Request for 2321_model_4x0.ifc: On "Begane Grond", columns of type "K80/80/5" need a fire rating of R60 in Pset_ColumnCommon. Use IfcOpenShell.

First a look at what the model holds.

```python
import ifcopenshell
import ifcopenshell.util.element

model = ifcopenshell.open("2321_model_4x0.ifc")
print(model.schema)
storey = next(s for s in model.by_type("IfcBuildingStorey") if s.Name == "Begane Grond")
columns = [e for e in ifcopenshell.util.element.get_decomposition(storey) if e.is_a("IfcColumn")]
seen = {}
for e in columns:
    element_type = ifcopenshell.util.element.get_type(e)
    key = (element_type.Name if element_type != e and element_type else None, ifcopenshell.util.element.get_pset(e, "Pset_ColumnCommon", "FireRating"))
    seen[key] = seen.get(key, 0) + 1
for (name, value), count in sorted(seen.items(), key=str):
    print(count, "x", name, "|", value)
```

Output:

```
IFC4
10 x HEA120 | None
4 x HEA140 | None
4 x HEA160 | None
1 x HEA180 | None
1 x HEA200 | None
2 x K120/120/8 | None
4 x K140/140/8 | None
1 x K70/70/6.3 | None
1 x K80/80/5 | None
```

```python
import ifcopenshell
import ifcopenshell.api.pset
import ifcopenshell.util.element

model = ifcopenshell.open("2321_model_4x0.ifc")

storey = next(s for s in model.by_type("IfcBuildingStorey") if s.Name == "Begane Grond")
columns = [e for e in ifcopenshell.util.element.get_decomposition(storey) if e.is_a("IfcColumn")]

count = 0
for e in columns:
    element_type = ifcopenshell.util.element.get_type(e)
    if element_type in (None, e) or element_type.Name != "K80/80/5":
        continue
    # add_pset returns the element's existing set when there is one.
    pset = ifcopenshell.api.pset.add_pset(model, product=e, name="Pset_ColumnCommon")
    ifcopenshell.api.pset.edit_pset(model, pset=pset, properties={"FireRating": "R60"})
    count += 1

print(count, "columns updated")

model.write("2321_model_4x0-out.ifc")
```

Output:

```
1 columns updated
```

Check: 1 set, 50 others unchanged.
